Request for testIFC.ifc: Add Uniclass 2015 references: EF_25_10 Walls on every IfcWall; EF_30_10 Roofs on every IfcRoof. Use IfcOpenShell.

First a look at what the model holds.

```python
import ifcopenshell

model = ifcopenshell.open("testIFC.ifc")
print(model.schema)
print("classifications:", [c.Name for c in model.by_type("IfcClassification")])
for ifc_class in ("IfcDoor", "IfcRoof", "IfcStair", "IfcWall", "IfcWindow"):
    print(ifc_class, len(model.by_type(ifc_class)))
```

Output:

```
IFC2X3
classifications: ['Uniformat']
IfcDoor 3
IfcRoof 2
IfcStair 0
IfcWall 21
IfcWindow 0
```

```python
import ifcopenshell
import ifcopenshell.api.classification

model = ifcopenshell.open("testIFC.ifc")

# IFC2X3 requires Source and Edition and has no link from the project to the system.
system = model.create_entity("IfcClassification", Source="NBS", Edition="2015", Name="Uniclass 2015")

codes = {
    "IfcWall": ("EF_25_10", "Walls"),
    "IfcRoof": ("EF_30_10", "Roofs"),
}
for ifc_class, (code, name) in codes.items():
    products = model.by_type(ifc_class)
    ifcopenshell.api.classification.add_reference(
        model, products=products, classification=system, identification=code, name=name
    )
    print(code, len(products))

model.write("testIFC_updated.ifc")
```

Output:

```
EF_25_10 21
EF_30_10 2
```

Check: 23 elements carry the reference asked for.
